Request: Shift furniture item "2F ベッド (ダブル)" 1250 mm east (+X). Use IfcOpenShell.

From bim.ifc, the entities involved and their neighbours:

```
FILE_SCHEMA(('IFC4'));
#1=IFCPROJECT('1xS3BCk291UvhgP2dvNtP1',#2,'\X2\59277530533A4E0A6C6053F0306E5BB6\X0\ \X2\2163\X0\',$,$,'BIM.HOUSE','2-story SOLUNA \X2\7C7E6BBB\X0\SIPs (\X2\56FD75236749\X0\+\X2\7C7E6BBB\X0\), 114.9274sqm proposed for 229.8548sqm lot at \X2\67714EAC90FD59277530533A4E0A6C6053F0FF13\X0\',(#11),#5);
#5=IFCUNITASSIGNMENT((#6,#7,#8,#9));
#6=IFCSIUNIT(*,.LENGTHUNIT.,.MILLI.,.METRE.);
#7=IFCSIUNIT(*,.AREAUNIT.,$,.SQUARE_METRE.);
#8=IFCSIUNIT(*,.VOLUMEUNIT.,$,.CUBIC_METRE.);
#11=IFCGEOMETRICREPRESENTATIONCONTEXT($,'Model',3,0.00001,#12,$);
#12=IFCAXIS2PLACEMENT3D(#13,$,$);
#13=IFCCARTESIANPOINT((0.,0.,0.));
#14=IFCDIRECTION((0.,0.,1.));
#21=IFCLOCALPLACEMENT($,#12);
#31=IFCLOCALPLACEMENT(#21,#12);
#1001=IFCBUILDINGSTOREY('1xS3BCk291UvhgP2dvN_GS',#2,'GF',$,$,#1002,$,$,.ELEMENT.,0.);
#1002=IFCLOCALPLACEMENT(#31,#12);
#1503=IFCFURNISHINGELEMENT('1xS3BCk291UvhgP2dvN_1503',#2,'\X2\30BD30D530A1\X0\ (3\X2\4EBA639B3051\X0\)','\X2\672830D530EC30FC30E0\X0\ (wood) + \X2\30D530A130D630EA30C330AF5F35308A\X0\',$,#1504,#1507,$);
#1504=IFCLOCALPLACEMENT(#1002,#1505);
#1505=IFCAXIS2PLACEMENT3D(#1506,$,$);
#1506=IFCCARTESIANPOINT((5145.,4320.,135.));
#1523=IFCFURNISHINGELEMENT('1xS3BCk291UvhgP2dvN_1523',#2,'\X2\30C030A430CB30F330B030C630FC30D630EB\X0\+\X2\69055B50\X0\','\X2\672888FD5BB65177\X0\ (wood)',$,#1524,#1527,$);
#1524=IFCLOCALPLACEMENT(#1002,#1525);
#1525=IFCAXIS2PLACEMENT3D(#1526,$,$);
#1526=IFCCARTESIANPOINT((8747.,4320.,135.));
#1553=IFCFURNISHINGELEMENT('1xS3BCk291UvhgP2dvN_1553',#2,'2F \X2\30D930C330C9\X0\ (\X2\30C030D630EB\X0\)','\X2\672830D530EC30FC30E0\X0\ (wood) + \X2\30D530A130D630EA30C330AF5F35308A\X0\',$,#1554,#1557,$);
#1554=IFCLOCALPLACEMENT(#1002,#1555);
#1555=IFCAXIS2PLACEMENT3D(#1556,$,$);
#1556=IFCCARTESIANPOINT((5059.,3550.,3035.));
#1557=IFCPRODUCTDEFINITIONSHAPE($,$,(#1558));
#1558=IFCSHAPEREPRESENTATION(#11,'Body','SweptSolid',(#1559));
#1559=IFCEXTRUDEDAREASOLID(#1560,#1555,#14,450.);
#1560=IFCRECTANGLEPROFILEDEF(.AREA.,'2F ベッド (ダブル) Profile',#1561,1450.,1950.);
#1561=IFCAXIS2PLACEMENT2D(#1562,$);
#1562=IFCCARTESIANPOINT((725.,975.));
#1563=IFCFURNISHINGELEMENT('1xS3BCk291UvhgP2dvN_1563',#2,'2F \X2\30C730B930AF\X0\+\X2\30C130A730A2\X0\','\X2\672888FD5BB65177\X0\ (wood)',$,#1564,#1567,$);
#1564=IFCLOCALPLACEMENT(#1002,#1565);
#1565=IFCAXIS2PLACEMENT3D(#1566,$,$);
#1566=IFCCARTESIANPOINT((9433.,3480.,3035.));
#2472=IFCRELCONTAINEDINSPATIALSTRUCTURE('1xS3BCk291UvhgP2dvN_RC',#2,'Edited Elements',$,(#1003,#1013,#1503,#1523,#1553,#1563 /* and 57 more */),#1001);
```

```python
import ifcopenshell
import ifcopenshell.api.geometry
import ifcopenshell.util.placement

model = ifcopenshell.open("bim.ifc")

item = model.by_id(1553)
matrix = ifcopenshell.util.placement.get_local_placement(item.ObjectPlacement)
matrix[0, 3] += 1250.0
ifcopenshell.api.geometry.edit_object_placement(model, product=item, matrix=matrix, is_si=False)

print(ifcopenshell.util.placement.get_local_placement(item.ObjectPlacement).round(3) + 0.0)

model.write("bim_edited.ifc")
```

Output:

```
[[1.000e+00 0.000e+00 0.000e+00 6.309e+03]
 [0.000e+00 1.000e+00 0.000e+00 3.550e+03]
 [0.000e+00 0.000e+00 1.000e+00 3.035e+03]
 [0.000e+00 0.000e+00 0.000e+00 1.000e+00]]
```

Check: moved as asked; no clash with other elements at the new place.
